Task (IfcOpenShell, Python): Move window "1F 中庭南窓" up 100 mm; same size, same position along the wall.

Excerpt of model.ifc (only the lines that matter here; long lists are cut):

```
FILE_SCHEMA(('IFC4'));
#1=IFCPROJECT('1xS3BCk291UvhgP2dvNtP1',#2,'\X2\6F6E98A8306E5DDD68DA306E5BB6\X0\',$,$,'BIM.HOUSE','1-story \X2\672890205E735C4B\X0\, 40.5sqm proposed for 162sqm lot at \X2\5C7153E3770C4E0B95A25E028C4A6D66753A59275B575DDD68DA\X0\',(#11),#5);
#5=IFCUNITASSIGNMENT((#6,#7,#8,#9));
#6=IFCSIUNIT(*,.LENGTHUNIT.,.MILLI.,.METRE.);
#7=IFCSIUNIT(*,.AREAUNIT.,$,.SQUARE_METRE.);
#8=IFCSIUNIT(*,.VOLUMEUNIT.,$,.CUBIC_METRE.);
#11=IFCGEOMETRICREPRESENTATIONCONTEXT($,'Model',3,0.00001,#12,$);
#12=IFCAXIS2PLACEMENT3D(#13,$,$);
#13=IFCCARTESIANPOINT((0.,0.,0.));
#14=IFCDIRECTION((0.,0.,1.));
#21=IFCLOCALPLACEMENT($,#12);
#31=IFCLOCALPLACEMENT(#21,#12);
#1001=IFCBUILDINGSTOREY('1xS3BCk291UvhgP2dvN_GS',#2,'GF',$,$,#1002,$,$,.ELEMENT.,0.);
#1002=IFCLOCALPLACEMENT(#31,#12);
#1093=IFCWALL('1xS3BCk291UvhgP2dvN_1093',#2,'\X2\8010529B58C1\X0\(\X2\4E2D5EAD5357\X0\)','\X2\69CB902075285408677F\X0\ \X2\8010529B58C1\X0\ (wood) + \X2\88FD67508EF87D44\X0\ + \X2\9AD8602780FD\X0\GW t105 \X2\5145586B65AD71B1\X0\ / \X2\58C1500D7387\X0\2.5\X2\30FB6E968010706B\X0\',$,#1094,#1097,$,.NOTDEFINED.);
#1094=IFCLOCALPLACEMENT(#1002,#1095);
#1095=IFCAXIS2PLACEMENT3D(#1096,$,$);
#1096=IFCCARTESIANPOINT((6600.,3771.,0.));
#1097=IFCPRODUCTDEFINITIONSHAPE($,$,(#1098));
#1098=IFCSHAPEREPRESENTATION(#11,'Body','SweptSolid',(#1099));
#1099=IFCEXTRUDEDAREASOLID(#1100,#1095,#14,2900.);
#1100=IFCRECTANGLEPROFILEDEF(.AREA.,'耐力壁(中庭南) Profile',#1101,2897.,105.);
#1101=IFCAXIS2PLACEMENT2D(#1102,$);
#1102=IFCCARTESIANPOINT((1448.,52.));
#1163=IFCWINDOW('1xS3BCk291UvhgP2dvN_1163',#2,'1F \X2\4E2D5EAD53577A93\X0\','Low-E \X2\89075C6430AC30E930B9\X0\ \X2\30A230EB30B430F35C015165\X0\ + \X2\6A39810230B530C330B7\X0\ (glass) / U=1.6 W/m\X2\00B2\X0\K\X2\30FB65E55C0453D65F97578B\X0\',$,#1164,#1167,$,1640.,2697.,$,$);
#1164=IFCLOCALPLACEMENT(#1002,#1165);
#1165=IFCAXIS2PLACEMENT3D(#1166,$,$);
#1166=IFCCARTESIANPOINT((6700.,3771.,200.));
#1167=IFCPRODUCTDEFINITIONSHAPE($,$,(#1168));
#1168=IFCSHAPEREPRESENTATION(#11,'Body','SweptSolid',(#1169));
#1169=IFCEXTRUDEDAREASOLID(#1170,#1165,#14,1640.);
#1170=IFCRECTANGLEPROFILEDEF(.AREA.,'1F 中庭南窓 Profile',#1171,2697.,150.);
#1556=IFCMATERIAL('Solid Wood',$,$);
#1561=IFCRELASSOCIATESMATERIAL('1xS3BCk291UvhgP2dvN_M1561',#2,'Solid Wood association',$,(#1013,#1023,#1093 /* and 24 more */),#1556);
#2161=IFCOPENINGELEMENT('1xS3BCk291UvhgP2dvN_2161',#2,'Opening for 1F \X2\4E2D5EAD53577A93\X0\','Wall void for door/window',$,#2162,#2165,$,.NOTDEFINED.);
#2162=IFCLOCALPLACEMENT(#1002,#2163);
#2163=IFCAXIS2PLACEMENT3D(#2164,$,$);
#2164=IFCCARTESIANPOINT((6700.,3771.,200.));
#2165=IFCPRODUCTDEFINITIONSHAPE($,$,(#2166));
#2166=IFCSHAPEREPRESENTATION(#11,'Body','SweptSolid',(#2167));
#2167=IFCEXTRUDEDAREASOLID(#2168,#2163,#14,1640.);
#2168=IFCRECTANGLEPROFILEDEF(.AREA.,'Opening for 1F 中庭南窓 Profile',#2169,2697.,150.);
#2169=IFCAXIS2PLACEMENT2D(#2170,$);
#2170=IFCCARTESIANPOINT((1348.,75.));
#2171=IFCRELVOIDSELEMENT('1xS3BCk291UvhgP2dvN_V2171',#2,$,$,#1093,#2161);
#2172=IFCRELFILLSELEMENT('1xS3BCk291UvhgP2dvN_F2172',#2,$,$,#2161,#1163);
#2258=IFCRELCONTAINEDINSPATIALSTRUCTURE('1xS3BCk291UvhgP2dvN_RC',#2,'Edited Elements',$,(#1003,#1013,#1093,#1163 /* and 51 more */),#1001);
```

```python
import numpy as np
import ifcopenshell
import ifcopenshell.api.geometry
import ifcopenshell.util.placement
import ifcopenshell.util.unit

model = ifcopenshell.open("model.ifc")
unit_scale = ifcopenshell.util.unit.calculate_unit_scale(model)

window = model.by_guid("1xS3BCk291UvhgP2dvN_1163")
opening = window.FillsVoids[0].RelatingOpeningElement
dz = 100.0

shift = np.array([0.0, 0.0, dz])
# The window is not placed relative to its opening, so move both.
for product in (opening, window):
    matrix = ifcopenshell.util.placement.get_local_placement(product.ObjectPlacement)
    matrix[:3, 3] += shift
    ifcopenshell.api.geometry.edit_object_placement(model, product=product, matrix=matrix, is_si=False)

print(f"moved by {dz * unit_scale:+.3f} m")

model.write("model_v2.ifc")
```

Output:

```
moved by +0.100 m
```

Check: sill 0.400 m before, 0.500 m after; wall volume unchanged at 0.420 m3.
